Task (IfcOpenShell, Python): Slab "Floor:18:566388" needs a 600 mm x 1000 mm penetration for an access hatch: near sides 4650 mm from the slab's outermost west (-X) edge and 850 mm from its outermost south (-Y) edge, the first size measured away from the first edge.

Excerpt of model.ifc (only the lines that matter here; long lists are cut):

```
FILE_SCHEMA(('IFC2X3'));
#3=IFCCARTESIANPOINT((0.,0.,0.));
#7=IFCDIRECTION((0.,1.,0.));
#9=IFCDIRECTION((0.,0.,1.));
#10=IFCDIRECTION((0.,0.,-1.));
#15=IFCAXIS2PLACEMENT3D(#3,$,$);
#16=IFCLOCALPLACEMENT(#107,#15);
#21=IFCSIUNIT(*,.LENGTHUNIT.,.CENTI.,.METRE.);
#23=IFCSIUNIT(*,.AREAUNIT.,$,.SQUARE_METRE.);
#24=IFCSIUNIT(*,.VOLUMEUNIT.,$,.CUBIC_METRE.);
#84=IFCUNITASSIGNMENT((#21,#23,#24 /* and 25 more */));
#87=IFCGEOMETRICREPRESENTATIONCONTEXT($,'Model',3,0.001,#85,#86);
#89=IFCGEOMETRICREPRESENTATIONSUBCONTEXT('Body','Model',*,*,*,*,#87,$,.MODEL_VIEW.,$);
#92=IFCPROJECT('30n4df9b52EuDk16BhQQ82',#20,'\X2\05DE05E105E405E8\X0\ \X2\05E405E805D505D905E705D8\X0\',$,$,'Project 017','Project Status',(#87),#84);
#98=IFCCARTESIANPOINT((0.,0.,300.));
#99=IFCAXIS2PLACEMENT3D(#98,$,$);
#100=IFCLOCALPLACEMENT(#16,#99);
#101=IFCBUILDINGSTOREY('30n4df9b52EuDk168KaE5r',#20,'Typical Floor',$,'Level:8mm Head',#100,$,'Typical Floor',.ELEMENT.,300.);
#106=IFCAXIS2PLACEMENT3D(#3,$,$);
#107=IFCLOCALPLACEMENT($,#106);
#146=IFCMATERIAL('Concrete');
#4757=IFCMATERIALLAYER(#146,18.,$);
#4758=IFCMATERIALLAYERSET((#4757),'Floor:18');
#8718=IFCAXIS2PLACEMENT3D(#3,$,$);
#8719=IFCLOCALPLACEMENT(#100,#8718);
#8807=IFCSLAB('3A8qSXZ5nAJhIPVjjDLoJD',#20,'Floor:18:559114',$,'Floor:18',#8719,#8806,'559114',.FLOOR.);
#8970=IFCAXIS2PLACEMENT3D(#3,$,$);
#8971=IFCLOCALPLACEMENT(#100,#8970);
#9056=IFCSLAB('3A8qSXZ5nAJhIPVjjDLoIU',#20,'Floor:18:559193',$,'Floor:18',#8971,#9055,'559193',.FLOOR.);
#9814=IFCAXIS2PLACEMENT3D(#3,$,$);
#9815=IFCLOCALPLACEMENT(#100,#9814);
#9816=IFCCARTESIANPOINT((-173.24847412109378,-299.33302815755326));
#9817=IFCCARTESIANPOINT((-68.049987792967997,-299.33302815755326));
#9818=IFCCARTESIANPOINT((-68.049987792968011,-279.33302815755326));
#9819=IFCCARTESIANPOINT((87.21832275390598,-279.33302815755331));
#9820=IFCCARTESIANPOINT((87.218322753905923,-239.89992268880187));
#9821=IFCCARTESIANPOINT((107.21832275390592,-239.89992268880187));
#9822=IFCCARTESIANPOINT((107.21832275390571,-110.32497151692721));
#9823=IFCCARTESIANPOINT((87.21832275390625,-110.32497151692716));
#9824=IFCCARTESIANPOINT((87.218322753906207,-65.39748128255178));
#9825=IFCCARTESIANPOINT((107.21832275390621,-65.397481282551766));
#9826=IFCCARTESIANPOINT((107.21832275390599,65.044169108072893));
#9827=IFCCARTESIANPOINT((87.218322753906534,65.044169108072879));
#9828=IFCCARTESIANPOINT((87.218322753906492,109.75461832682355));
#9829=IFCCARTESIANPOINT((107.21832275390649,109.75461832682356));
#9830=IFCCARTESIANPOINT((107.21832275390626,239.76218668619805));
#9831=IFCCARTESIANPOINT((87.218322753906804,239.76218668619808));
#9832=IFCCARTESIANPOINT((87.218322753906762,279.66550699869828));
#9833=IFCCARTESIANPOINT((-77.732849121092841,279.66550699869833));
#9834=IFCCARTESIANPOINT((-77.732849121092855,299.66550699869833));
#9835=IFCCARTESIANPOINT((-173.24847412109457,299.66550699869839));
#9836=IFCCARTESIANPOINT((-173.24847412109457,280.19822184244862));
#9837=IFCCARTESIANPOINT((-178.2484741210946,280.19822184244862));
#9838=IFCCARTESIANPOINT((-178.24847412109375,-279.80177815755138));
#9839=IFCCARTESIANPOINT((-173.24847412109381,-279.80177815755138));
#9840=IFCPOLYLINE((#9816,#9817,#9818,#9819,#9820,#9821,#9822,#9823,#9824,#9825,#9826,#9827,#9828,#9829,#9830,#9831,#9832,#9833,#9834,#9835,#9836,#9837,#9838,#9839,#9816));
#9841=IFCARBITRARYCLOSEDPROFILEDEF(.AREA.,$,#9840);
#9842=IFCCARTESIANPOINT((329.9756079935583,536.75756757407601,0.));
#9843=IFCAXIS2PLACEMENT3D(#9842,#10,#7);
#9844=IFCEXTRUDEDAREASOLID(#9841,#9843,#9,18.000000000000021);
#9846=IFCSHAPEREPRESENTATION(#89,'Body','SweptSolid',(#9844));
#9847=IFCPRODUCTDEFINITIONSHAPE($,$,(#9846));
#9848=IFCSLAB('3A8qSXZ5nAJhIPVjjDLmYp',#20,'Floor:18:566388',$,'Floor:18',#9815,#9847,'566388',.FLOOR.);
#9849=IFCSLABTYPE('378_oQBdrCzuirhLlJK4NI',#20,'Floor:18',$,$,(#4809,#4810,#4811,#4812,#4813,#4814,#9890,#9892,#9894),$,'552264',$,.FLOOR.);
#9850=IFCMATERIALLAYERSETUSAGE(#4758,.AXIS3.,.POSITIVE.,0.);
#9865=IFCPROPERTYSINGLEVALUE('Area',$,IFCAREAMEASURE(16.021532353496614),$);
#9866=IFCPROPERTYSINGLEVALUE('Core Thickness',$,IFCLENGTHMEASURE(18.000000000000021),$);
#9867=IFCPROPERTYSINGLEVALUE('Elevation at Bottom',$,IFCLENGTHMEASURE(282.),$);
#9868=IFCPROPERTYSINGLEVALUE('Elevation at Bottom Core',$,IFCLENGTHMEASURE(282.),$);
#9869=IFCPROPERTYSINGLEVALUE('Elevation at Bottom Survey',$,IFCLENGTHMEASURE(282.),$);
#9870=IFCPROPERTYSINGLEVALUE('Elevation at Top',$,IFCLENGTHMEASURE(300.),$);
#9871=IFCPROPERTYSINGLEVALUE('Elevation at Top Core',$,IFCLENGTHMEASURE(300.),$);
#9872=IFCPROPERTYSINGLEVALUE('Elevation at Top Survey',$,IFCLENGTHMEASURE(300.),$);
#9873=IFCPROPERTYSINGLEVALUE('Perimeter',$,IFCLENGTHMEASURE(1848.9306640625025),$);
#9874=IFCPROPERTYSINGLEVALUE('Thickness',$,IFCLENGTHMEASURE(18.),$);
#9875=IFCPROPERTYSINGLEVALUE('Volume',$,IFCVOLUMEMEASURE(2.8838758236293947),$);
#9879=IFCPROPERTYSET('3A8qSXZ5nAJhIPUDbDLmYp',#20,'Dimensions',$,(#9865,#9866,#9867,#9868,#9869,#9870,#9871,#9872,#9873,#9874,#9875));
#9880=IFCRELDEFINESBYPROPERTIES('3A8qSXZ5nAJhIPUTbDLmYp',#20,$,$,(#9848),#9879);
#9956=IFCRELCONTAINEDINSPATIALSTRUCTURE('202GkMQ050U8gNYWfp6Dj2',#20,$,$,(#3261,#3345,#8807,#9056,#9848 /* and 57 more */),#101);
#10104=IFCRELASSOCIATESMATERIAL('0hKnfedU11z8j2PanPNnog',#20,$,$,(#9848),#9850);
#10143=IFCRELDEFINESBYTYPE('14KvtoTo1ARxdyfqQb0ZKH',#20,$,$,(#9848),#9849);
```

```python
import numpy as np
import ifcopenshell
import ifcopenshell.api.feature
import ifcopenshell.api.geometry
import ifcopenshell.api.pset
import ifcopenshell.api.root
import ifcopenshell.geom
import ifcopenshell.util.element
import ifcopenshell.util.placement
import ifcopenshell.util.representation
import ifcopenshell.util.shape
import ifcopenshell.util.unit

model = ifcopenshell.open("model.ifc")
unit_scale = ifcopenshell.util.unit.calculate_unit_scale(model)
area_scale = ifcopenshell.util.unit.calculate_unit_scale(model, "AREAUNIT")
volume_scale = ifcopenshell.util.unit.calculate_unit_scale(model, "VOLUMEUNIT")
settings = ifcopenshell.geom.settings()


def volume(element):
    """Net volume in cubic metres, openings subtracted."""
    shape = ifcopenshell.geom.create_shape(settings, element)
    return ifcopenshell.util.shape.get_volume(shape.geometry)


slab = model.by_guid("3A8qSXZ5nAJhIPVjjDLmYp")
before = volume(slab)

# Extent in the slab's own axes, in metres. The edges named are its -X and -Y sides.
slab_shape = ifcopenshell.geom.create_shape(settings, slab)
vertices = ifcopenshell.util.shape.get_vertices(slab_shape.geometry)
x_min, y_min, bottom = vertices.min(axis=0)
top = vertices[:, 2].max()

opening = ifcopenshell.api.root.create_entity(model, ifc_class="IfcOpeningElement", name="Access hatch opening")
context = ifcopenshell.util.representation.get_context(model, "Model", "Body", "MODEL_VIEW")
width, depth = 0.6, 1
outline = [(0.0, 0.0), (width, 0.0), (width, depth), (0.0, depth), (0.0, 0.0)]
# Overshoot both faces by 50 mm so the cut is clean.
shape = ifcopenshell.api.geometry.add_slab_representation(
    model, context=context, depth=top - bottom + 0.1, polyline=outline
)
ifcopenshell.api.geometry.assign_representation(model, product=opening, representation=shape)

matrix = ifcopenshell.util.placement.get_local_placement(slab.ObjectPlacement)
matrix[:, 3] = matrix @ np.append(np.array([x_min + 4.65, y_min + 0.85, bottom - 0.05]) / unit_scale, 1.0)
ifcopenshell.api.geometry.edit_object_placement(model, product=opening, matrix=matrix, is_si=False)
ifcopenshell.api.feature.add_feature(model, feature=opening, element=slab)

after = volume(slab)

# Update the slab's stored quantities.
pset = model.by_id(ifcopenshell.util.element.get_pset(slab, "Dimensions", should_inherit=False)["id"])
ifcopenshell.api.pset.edit_pset(model, pset=pset, properties={
    "Area": model.create_entity("IfcAreaMeasure", after / (top - bottom) / area_scale),
    "Volume": model.create_entity("IfcVolumeMeasure", after / volume_scale),
})

print(f"slab volume {before:.3f} -> {after:.3f} m3")

model.write("model-out.ifc")
```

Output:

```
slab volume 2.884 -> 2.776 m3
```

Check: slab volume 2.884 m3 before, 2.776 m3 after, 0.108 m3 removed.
